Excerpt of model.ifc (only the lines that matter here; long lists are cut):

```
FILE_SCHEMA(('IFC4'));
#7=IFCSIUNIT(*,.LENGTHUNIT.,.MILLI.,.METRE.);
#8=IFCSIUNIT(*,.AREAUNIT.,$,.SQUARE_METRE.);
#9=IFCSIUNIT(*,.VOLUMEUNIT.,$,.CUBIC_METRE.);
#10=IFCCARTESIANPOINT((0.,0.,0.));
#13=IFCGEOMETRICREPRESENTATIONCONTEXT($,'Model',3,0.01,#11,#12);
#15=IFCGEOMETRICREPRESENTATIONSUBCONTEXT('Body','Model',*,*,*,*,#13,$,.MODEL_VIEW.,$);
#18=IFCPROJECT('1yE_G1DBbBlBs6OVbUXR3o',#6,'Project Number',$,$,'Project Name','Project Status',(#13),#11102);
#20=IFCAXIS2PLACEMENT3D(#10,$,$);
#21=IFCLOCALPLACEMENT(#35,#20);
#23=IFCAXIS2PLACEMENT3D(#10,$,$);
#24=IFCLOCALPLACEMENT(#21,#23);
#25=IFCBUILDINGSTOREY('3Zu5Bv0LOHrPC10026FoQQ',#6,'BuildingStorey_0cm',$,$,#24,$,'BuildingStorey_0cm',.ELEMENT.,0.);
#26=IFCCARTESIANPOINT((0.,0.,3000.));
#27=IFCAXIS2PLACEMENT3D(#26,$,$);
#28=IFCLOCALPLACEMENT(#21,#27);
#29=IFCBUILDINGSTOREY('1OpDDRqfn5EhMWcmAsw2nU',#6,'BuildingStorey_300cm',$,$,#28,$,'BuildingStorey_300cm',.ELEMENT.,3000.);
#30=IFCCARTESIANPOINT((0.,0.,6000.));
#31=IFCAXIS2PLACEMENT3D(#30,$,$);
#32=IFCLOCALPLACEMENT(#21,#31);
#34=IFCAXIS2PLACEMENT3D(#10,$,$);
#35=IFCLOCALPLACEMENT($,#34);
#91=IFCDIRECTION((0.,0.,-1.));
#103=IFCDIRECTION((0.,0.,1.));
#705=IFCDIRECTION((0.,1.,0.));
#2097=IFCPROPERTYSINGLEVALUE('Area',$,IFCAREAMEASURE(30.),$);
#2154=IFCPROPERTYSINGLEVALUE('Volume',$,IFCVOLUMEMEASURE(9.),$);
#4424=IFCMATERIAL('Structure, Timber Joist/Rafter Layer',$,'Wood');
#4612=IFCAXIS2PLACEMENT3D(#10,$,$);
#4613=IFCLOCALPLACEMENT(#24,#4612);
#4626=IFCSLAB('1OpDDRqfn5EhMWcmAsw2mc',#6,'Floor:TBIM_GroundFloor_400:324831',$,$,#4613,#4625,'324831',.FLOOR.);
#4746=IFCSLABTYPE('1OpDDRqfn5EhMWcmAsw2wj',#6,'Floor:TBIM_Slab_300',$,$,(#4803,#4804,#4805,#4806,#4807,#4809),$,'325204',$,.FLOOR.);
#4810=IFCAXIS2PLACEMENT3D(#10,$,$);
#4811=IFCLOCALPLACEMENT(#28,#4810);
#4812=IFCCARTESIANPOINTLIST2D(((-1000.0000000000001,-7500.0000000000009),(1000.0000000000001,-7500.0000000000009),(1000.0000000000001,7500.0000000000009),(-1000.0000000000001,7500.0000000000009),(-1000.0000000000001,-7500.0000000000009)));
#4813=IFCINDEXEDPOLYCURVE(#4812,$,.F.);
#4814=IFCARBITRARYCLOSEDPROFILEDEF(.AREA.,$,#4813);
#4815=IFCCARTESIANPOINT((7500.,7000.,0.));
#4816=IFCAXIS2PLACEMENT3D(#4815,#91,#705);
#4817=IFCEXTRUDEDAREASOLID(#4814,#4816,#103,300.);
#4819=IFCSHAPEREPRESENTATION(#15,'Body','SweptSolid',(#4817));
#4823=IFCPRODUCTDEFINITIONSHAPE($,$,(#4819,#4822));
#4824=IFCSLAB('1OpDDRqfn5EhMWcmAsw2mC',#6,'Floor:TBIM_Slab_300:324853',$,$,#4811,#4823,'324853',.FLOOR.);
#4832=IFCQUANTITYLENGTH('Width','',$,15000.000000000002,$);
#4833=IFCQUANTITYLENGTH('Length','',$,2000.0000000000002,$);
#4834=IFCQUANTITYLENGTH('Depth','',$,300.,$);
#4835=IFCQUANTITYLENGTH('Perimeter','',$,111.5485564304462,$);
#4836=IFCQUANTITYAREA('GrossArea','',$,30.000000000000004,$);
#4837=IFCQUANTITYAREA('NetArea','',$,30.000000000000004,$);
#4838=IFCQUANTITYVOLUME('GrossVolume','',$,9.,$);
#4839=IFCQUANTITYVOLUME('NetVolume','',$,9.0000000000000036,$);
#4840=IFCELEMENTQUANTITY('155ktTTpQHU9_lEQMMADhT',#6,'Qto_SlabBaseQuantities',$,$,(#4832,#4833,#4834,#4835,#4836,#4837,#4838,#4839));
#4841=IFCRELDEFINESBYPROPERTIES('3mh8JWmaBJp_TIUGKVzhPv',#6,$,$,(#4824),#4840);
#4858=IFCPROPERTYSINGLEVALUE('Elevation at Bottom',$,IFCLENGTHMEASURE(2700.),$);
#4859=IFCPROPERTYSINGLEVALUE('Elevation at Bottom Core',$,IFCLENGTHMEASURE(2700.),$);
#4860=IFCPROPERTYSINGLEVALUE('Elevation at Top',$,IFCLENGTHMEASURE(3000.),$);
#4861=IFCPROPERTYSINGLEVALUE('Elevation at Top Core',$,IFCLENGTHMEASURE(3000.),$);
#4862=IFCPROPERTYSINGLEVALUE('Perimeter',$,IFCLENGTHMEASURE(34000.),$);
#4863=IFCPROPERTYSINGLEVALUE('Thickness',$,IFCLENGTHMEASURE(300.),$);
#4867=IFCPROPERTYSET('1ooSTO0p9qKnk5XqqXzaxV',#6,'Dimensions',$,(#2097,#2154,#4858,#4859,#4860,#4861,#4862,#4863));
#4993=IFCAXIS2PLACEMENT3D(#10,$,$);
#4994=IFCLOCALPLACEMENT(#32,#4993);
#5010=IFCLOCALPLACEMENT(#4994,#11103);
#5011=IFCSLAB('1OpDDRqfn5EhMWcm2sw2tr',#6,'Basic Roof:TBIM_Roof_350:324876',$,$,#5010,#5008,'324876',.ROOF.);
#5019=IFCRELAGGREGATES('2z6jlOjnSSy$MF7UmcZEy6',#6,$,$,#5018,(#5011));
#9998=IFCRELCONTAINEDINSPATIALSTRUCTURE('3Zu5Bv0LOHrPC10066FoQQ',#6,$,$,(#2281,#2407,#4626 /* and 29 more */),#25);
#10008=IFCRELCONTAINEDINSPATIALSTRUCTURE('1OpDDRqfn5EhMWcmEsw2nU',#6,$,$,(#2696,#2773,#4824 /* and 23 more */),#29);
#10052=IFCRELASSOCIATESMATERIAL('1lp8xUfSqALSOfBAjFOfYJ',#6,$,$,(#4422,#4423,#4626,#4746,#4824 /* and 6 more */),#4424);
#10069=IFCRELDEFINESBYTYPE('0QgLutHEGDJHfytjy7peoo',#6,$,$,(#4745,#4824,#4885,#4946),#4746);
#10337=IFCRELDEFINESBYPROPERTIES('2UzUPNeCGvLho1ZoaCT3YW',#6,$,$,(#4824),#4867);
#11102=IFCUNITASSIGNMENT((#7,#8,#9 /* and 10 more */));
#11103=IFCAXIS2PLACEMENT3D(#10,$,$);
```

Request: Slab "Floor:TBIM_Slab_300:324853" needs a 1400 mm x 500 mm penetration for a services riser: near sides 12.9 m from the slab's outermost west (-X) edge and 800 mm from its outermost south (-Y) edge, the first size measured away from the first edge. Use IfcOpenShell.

```python
import numpy as np
import ifcopenshell
import ifcopenshell.api.feature
import ifcopenshell.api.geometry
import ifcopenshell.api.pset
import ifcopenshell.api.root
import ifcopenshell.geom
import ifcopenshell.util.element
import ifcopenshell.util.placement
import ifcopenshell.util.representation
import ifcopenshell.util.shape
import ifcopenshell.util.unit

model = ifcopenshell.open("model.ifc")
unit_scale = ifcopenshell.util.unit.calculate_unit_scale(model)
area_scale = ifcopenshell.util.unit.calculate_unit_scale(model, "AREAUNIT")
volume_scale = ifcopenshell.util.unit.calculate_unit_scale(model, "VOLUMEUNIT")
settings = ifcopenshell.geom.settings()


def volume(element):
    """Net volume in cubic metres, openings subtracted."""
    shape = ifcopenshell.geom.create_shape(settings, element)
    return ifcopenshell.util.shape.get_volume(shape.geometry)


slab = model.by_guid("1OpDDRqfn5EhMWcmAsw2mC")
before = volume(slab)

# Extent in the slab's own axes, in metres. The edges named are its -X and -Y sides.
slab_shape = ifcopenshell.geom.create_shape(settings, slab)
vertices = ifcopenshell.util.shape.get_vertices(slab_shape.geometry)
x_min, y_min, bottom = vertices.min(axis=0)
top = vertices[:, 2].max()

opening = ifcopenshell.api.root.create_entity(model, ifc_class="IfcOpeningElement", name="Services riser opening", predefined_type="OPENING")
context = ifcopenshell.util.representation.get_context(model, "Model", "Body", "MODEL_VIEW")
width, depth = 1.4, 0.5
outline = [(0.0, 0.0), (width, 0.0), (width, depth), (0.0, depth), (0.0, 0.0)]
# Overshoot both faces by 50 mm so the cut is clean.
shape = ifcopenshell.api.geometry.add_slab_representation(
    model, context=context, depth=top - bottom + 0.1, polyline=outline
)
ifcopenshell.api.geometry.assign_representation(model, product=opening, representation=shape)

matrix = ifcopenshell.util.placement.get_local_placement(slab.ObjectPlacement)
matrix[:, 3] = matrix @ np.append(np.array([x_min + 12.9, y_min + 0.8, bottom - 0.05]) / unit_scale, 1.0)
ifcopenshell.api.geometry.edit_object_placement(model, product=opening, matrix=matrix, is_si=False)
ifcopenshell.api.feature.add_feature(model, feature=opening, element=slab)

after = volume(slab)

# Update the slab's stored quantities.
qto = model.by_id(ifcopenshell.util.element.get_pset(slab, "Qto_SlabBaseQuantities", should_inherit=False)["id"])
ifcopenshell.api.pset.edit_qto(model, qto=qto, properties={
    "NetArea": after / (top - bottom) / area_scale,
    "NetVolume": after / volume_scale,
})
pset = model.by_id(ifcopenshell.util.element.get_pset(slab, "Dimensions", should_inherit=False)["id"])
ifcopenshell.api.pset.edit_pset(model, pset=pset, properties={
    "Area": model.create_entity("IfcAreaMeasure", after / (top - bottom) / area_scale),
    "Volume": model.create_entity("IfcVolumeMeasure", after / volume_scale),
})

print(f"slab volume {before:.3f} -> {after:.3f} m3")

model.write("model_v2.ifc")
```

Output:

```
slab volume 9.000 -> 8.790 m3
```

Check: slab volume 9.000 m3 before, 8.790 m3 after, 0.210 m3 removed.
